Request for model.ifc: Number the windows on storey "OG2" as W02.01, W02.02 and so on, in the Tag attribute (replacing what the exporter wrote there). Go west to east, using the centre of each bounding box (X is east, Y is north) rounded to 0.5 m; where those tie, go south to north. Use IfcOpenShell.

First a look at what the model holds.

```python
import ifcopenshell
import ifcopenshell.util.element
import ifcopenshell.util.placement

model = ifcopenshell.open("model.ifc")
print(model.schema)
storey = next(s for s in model.by_type("IfcBuildingStorey") if s.Name == "OG2")
windows = [e for e in ifcopenshell.util.element.get_decomposition(storey) if e.is_a("IfcWindow")]
for e in sorted(windows, key=lambda e: e.id()):
    origin = ifcopenshell.util.placement.get_local_placement(e.ObjectPlacement)[:3, 3]
    print(e.id(), e.Tag, e.Name, origin.round(2) + 0.0, sep=" | ")
```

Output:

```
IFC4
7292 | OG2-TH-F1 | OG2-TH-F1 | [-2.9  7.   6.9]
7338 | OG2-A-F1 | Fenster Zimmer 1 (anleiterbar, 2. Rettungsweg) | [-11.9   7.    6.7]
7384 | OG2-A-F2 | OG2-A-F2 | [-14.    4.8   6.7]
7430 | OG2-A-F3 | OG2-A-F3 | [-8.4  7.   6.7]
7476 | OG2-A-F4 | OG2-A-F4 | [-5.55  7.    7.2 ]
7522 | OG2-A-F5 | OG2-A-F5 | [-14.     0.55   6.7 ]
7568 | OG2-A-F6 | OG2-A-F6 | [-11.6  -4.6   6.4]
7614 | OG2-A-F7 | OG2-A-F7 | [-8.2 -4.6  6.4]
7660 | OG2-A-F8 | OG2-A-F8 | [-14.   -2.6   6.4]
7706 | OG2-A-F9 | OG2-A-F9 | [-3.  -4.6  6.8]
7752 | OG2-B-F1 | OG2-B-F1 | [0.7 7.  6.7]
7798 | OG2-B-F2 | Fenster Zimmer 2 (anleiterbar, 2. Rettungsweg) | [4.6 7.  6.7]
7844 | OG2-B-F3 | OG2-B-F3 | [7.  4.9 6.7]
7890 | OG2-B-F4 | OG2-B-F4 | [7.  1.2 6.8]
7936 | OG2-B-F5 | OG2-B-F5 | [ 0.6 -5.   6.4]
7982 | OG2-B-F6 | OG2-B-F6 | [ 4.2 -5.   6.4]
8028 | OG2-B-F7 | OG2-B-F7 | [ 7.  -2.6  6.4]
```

```python
import ifcopenshell
import ifcopenshell.geom
import ifcopenshell.util.element
import ifcopenshell.util.shape

model = ifcopenshell.open("model.ifc")
settings = ifcopenshell.geom.settings()
settings.set("use-world-coords", True)


def centre(element):
    shape = ifcopenshell.geom.create_shape(settings, element)
    return ifcopenshell.util.shape.get_bbox_centroid(shape.geometry)


storey = next(s for s in model.by_type("IfcBuildingStorey") if s.Name == "OG2")
windows = [e for e in ifcopenshell.util.element.get_decomposition(storey) if e.is_a("IfcWindow")]

# Insertion points can sit at a corner or the storey origin, so sort by the geometry (in metres).
centres = {e: centre(e) for e in windows}
windows.sort(key=lambda e: (round(centres[e][0] / 0.5), centres[e][1]))

for i, e in enumerate(windows, start=1):
    number = f"W02.{i:02d}"
    e.Tag = number
    print(e.id(), number)

model.write("model-out.ifc")
```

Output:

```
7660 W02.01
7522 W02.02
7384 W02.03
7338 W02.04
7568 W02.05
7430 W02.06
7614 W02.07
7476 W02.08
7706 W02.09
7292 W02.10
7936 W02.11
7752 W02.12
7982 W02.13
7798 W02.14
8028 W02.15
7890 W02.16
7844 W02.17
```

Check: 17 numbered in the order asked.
